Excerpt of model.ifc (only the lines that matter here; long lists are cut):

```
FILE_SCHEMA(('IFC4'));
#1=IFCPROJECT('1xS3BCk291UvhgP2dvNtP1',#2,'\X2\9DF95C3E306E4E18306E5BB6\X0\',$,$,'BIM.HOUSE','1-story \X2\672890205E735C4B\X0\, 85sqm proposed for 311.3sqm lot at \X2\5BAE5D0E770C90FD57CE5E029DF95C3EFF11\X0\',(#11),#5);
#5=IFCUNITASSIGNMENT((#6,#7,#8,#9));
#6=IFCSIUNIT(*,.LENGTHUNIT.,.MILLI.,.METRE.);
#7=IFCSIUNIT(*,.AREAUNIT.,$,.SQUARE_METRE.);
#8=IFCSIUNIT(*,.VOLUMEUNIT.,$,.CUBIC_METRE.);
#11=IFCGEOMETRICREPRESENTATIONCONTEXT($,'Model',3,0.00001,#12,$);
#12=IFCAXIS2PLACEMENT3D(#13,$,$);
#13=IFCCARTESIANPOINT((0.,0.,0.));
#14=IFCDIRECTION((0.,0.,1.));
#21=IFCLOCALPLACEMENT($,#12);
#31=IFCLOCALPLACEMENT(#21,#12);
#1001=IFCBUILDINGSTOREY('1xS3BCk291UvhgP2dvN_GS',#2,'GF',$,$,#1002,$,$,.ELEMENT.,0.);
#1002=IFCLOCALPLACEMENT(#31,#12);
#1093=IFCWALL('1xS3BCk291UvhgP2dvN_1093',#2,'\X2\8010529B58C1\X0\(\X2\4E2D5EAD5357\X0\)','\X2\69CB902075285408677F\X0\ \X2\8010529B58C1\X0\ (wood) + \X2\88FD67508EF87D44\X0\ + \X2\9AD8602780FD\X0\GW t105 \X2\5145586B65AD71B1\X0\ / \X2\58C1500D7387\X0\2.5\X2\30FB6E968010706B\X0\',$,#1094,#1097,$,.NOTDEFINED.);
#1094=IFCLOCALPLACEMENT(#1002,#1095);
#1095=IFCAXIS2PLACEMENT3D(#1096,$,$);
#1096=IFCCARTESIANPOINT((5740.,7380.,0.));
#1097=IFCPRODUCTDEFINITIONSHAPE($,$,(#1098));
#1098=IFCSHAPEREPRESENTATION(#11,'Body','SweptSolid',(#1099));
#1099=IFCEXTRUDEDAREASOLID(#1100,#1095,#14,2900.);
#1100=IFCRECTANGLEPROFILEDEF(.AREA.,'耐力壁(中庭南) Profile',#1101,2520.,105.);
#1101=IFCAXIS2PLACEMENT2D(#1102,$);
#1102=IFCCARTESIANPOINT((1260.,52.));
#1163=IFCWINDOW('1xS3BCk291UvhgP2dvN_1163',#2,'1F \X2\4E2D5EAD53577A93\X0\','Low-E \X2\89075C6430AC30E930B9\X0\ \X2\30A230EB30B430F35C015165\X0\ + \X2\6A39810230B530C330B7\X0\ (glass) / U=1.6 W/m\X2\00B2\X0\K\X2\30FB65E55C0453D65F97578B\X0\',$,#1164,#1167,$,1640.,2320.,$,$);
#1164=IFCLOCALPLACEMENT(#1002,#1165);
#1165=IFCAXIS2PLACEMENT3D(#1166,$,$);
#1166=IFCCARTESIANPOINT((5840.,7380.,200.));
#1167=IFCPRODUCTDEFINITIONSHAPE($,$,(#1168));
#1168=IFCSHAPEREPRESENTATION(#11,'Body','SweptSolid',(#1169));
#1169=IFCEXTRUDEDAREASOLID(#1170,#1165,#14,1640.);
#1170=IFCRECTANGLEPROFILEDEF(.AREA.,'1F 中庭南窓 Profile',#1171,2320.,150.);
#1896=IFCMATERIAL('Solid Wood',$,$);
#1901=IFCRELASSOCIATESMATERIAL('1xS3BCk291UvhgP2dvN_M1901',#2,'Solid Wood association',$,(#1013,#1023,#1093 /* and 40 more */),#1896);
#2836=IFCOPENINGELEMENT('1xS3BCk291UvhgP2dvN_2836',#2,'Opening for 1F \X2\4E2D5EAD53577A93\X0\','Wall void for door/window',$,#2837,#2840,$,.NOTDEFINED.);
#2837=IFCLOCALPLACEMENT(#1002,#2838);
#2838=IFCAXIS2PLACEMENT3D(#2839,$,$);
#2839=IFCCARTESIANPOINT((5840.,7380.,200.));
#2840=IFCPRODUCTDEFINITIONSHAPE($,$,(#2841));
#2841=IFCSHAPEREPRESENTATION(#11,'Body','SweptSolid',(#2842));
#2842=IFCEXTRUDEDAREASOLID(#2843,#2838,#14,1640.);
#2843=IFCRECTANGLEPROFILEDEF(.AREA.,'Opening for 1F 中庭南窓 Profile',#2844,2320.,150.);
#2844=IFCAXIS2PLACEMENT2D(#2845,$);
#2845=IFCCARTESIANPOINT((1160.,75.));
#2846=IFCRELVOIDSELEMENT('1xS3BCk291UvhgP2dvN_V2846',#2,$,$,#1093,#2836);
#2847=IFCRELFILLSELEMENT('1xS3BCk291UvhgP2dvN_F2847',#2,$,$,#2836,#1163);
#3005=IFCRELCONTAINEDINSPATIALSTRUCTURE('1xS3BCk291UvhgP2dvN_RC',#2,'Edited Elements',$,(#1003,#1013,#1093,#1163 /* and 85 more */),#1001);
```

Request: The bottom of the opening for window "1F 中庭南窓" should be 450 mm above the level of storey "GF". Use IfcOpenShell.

```python
import numpy as np
import ifcopenshell
import ifcopenshell.api.geometry
import ifcopenshell.geom
import ifcopenshell.util.element
import ifcopenshell.util.placement
import ifcopenshell.util.shape
import ifcopenshell.util.unit

model = ifcopenshell.open("model.ifc")
unit_scale = ifcopenshell.util.unit.calculate_unit_scale(model)

window = model.by_guid("1xS3BCk291UvhgP2dvN_1163")
opening = window.FillsVoids[0].RelatingOpeningElement
storey = ifcopenshell.util.element.get_container(window, ifc_class="IfcBuildingStorey")
level = ifcopenshell.util.placement.get_local_placement(storey.ObjectPlacement)[2, 3]

# The opening's origin need not be at the sill, so measure its lowest point.
shape = ifcopenshell.geom.create_shape(ifcopenshell.geom.settings(), opening)
bottom = ifcopenshell.util.shape.get_shape_bottom_elevation(shape, shape.geometry) / unit_scale
dz = level + 0.45 / unit_scale - bottom

shift = np.array([0.0, 0.0, dz])
# The window is not placed relative to its opening, so move both.
for product in (opening, window):
    matrix = ifcopenshell.util.placement.get_local_placement(product.ObjectPlacement)
    matrix[:3, 3] += shift
    ifcopenshell.api.geometry.edit_object_placement(model, product=product, matrix=matrix, is_si=False)

print(f"moved by {dz * unit_scale:+.3f} m")

model.write("model-out.ifc")
```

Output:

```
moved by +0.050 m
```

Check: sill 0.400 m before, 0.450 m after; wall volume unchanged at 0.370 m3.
